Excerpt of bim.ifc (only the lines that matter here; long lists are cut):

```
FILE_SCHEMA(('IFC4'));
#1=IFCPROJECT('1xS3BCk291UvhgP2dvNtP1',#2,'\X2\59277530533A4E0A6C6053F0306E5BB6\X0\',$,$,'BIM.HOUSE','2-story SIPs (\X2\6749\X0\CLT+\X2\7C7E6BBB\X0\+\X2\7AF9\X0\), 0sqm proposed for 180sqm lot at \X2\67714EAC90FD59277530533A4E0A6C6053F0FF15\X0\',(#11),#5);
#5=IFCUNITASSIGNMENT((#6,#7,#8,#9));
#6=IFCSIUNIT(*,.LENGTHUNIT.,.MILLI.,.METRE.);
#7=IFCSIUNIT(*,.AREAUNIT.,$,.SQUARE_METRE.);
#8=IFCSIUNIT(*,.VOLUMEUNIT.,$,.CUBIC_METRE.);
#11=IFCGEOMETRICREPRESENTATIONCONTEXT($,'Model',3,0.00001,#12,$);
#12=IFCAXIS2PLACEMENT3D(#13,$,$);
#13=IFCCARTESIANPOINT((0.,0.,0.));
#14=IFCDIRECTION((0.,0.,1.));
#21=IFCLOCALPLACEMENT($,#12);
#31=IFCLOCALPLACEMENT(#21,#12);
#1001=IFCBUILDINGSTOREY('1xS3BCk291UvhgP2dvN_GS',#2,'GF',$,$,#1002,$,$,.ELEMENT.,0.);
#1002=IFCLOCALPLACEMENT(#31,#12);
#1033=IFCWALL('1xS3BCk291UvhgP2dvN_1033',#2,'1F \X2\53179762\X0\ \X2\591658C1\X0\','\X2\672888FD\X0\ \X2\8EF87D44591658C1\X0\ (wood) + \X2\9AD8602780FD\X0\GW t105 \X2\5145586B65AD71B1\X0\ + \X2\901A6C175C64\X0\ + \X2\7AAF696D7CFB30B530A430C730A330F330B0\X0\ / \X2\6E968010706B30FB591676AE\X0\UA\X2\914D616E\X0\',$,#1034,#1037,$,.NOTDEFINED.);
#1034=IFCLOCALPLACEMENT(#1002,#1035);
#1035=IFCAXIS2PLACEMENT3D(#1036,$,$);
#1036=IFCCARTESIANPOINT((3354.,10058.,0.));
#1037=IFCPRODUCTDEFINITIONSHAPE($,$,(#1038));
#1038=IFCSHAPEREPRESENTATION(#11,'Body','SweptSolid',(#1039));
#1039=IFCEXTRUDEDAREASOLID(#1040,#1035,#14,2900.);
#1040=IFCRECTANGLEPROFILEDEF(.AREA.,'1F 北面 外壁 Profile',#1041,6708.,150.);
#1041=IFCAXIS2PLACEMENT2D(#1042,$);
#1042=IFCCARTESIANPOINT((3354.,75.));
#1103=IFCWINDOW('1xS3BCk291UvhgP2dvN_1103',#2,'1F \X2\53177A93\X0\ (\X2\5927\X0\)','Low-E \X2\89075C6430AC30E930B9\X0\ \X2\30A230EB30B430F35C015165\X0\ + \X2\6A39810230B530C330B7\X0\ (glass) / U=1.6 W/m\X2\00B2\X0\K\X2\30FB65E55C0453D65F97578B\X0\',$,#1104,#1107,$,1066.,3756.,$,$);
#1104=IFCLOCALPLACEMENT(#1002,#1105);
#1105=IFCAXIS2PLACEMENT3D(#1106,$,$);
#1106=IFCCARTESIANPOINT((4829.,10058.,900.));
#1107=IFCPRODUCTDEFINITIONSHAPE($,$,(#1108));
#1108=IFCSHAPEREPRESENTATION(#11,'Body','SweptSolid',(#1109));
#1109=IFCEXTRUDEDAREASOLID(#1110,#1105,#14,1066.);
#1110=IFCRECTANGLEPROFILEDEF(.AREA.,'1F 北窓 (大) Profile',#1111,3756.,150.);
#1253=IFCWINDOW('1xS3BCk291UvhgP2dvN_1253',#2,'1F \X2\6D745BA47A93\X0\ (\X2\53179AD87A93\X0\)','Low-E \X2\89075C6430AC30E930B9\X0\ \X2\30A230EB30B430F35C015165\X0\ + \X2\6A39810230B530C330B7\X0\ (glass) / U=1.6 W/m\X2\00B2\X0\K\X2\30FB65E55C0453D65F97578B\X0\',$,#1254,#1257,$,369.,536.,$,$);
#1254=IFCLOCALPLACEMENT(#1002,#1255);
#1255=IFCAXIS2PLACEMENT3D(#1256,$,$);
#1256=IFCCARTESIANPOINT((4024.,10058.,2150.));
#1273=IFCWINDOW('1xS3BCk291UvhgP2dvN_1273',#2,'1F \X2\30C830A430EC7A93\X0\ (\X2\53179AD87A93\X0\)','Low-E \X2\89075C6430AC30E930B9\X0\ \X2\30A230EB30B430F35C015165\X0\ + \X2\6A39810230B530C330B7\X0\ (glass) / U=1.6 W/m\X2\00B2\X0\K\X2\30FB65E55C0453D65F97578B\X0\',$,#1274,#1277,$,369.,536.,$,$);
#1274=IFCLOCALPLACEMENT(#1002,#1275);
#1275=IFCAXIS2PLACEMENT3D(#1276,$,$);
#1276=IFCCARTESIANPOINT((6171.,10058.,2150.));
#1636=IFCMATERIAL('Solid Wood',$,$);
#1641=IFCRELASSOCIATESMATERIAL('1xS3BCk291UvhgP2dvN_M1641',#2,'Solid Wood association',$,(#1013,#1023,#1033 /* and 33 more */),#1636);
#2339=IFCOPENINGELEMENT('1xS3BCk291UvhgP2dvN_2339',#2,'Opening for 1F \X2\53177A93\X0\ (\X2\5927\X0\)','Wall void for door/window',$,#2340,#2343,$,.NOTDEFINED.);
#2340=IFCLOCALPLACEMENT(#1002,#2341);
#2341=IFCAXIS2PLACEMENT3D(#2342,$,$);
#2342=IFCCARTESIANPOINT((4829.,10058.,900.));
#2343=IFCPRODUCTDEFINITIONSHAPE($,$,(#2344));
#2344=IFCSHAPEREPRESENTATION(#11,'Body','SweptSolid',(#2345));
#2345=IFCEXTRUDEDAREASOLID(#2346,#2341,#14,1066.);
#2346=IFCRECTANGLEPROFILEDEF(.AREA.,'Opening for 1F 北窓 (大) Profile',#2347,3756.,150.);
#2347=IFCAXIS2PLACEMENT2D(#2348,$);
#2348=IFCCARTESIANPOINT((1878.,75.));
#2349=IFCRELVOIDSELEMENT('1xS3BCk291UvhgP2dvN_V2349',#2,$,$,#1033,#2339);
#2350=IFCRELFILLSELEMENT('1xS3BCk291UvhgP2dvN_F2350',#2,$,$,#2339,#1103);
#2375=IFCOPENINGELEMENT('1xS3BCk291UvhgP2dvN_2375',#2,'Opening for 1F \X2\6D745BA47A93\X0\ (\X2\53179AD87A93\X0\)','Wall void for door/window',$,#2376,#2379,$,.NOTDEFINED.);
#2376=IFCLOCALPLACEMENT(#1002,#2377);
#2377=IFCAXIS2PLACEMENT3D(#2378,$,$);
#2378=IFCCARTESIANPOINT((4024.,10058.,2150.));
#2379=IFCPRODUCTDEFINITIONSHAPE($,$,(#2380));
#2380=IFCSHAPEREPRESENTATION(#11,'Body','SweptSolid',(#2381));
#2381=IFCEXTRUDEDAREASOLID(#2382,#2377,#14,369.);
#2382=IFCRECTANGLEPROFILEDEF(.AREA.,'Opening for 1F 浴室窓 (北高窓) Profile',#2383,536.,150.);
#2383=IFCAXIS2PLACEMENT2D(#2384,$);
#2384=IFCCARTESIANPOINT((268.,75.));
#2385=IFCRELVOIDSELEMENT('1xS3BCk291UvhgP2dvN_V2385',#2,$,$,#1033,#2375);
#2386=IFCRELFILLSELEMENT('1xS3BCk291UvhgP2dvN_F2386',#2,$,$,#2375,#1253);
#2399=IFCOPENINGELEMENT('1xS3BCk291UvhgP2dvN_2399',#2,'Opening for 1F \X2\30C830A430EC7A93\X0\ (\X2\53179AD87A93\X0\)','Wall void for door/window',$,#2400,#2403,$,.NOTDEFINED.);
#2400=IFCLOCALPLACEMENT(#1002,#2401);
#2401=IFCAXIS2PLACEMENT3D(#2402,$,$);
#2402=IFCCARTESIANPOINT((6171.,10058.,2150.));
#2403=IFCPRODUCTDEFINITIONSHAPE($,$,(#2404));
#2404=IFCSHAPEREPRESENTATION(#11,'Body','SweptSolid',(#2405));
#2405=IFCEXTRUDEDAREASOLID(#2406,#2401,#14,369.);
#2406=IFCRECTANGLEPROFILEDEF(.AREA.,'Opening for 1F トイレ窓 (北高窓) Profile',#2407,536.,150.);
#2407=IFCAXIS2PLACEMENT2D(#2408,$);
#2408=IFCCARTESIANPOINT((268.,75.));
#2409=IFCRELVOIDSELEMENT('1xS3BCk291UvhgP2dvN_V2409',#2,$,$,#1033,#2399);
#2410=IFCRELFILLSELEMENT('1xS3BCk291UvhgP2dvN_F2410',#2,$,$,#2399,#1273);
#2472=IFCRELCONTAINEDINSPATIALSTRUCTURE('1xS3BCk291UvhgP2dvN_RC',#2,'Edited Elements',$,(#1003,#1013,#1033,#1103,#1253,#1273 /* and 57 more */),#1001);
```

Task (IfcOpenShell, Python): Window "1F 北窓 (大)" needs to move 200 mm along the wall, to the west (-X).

```python
import ifcopenshell
import ifcopenshell.api.geometry
import ifcopenshell.util.placement
import ifcopenshell.util.unit

model = ifcopenshell.open("bim.ifc")
unit_scale = ifcopenshell.util.unit.calculate_unit_scale(model)

window = model.by_guid("1xS3BCk291UvhgP2dvN_1103")
opening = window.FillsVoids[0].RelatingOpeningElement
wall = opening.VoidsElements[0].RelatingBuildingElement

wall_matrix = ifcopenshell.util.placement.get_local_placement(wall.ObjectPlacement)
shift = wall_matrix[:3, 0] * -0.2 / unit_scale
before = ifcopenshell.util.placement.get_local_placement(window.ObjectPlacement)[:3, 3].copy()

# The window is not placed relative to its opening, so move both.
for product in (opening, window):
    matrix = ifcopenshell.util.placement.get_local_placement(product.ObjectPlacement)
    matrix[:3, 3] += shift
    ifcopenshell.api.geometry.edit_object_placement(model, product=product, matrix=matrix, is_si=False)

after = ifcopenshell.util.placement.get_local_placement(window.ObjectPlacement)[:3, 3]
print("window moved by", (after - before).round(3) + 0.0)

model.write("bim_edited.ifc")
```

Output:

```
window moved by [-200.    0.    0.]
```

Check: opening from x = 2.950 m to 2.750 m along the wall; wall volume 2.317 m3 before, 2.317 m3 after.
